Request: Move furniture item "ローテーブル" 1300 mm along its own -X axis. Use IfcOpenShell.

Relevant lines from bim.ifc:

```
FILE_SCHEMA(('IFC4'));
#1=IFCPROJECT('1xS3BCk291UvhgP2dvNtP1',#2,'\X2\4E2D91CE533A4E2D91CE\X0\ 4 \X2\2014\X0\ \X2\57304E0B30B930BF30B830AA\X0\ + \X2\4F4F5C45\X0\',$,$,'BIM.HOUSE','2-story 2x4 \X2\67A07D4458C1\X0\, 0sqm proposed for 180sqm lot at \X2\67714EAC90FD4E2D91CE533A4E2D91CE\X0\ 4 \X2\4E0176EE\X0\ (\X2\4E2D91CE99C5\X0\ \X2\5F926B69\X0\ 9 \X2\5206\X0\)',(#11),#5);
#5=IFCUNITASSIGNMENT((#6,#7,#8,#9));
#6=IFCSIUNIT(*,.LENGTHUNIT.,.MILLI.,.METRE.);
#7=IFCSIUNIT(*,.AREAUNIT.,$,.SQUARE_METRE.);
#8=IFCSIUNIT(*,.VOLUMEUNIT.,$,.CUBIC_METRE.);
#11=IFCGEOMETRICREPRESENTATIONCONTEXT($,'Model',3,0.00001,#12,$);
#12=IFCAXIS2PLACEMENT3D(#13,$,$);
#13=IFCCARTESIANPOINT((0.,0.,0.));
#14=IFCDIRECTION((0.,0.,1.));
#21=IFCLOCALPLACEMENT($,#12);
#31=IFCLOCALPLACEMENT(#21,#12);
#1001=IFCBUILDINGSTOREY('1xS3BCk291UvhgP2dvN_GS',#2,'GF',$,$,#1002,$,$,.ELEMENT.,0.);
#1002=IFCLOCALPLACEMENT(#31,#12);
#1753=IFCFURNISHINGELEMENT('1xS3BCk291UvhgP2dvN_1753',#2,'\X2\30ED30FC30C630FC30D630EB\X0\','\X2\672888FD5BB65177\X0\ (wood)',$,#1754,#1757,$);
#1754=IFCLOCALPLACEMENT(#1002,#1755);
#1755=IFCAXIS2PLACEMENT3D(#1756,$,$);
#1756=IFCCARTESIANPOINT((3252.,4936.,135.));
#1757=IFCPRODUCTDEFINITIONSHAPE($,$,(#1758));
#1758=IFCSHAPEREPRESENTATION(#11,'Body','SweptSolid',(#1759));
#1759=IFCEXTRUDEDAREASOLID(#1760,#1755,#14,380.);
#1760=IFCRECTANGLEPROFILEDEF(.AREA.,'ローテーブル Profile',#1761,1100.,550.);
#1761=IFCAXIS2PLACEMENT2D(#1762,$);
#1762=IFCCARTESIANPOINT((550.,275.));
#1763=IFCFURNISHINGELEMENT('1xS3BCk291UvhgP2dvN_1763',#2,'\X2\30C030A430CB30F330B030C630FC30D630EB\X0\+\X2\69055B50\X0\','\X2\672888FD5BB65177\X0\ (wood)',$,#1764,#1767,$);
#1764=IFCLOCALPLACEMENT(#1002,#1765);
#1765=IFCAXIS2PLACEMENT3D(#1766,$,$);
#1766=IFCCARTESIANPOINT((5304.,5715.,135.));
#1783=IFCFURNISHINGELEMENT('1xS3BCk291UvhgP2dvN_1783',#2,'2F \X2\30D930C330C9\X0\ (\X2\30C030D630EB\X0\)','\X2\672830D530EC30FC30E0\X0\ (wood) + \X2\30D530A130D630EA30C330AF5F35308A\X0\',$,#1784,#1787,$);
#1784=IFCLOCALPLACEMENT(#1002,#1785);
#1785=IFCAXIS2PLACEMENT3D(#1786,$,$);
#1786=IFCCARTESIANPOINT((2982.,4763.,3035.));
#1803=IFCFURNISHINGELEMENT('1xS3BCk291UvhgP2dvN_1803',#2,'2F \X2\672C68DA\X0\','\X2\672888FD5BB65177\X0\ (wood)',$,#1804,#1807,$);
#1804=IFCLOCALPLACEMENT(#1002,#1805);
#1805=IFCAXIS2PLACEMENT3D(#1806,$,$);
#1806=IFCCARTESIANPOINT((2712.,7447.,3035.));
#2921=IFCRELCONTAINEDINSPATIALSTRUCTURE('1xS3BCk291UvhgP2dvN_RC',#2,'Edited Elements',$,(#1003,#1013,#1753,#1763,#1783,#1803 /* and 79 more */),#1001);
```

```python
import ifcopenshell
import ifcopenshell.api.geometry
import ifcopenshell.util.placement

model = ifcopenshell.open("bim.ifc")

item = model.by_id(1753)
matrix = ifcopenshell.util.placement.get_local_placement(item.ObjectPlacement)
matrix[:3, 3] -= matrix[:3, 0] * 1300.0
ifcopenshell.api.geometry.edit_object_placement(model, product=item, matrix=matrix, is_si=False)

print(ifcopenshell.util.placement.get_local_placement(item.ObjectPlacement).round(3) + 0.0)

model.write("bim_edited.ifc")
```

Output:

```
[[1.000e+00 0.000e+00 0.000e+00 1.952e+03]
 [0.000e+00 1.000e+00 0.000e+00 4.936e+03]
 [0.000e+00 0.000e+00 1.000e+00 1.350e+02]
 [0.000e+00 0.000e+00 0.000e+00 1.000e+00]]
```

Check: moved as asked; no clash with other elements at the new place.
